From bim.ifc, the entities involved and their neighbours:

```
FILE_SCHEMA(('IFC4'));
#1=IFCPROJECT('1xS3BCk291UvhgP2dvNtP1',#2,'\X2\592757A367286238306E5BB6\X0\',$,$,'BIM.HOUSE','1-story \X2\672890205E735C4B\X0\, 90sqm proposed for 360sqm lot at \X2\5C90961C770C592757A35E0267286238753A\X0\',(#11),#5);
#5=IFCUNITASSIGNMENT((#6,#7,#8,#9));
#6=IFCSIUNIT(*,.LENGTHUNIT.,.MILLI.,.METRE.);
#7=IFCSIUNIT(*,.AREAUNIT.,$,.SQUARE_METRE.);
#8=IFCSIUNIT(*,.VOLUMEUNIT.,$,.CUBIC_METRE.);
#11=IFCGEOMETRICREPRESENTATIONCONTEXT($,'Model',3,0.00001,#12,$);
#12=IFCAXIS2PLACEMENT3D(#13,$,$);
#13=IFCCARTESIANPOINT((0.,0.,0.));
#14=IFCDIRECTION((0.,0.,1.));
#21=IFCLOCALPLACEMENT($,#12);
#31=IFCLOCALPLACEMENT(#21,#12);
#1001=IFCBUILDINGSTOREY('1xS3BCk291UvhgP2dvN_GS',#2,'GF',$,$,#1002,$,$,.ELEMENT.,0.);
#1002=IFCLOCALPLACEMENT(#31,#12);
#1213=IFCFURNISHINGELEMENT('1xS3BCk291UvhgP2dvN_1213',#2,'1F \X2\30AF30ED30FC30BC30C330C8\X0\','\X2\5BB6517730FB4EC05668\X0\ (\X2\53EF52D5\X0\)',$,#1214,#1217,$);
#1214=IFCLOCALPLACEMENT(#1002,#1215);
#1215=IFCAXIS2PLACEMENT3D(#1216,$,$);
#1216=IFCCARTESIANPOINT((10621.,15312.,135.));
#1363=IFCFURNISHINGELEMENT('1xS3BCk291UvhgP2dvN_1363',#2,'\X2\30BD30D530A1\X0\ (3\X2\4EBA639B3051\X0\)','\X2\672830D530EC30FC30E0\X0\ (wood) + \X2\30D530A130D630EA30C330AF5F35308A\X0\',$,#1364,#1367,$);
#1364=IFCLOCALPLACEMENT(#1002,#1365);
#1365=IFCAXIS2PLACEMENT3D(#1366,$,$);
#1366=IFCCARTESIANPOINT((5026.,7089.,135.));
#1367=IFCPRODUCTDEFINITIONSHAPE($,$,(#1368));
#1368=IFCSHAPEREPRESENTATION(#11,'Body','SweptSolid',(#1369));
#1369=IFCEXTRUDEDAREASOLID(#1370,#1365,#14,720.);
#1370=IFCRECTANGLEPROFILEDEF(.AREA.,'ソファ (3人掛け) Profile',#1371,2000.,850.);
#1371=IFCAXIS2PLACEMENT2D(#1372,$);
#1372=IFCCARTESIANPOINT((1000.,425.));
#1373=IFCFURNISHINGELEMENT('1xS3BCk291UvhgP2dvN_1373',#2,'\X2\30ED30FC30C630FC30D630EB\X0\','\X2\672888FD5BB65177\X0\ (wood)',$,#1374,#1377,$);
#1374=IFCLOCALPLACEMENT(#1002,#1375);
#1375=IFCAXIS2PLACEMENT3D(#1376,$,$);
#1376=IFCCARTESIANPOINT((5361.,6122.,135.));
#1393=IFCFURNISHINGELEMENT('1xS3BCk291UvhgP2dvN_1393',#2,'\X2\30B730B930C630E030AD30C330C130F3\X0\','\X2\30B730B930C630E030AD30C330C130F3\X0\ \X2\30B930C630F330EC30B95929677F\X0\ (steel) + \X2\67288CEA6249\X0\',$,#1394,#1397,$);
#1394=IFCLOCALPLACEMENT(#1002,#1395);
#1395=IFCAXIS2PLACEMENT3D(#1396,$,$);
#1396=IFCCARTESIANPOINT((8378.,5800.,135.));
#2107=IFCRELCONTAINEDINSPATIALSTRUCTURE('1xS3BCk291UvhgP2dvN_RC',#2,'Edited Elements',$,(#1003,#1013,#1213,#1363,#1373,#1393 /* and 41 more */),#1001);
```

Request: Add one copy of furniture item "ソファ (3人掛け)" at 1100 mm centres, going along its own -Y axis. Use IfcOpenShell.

```python
import ifcopenshell
import ifcopenshell.api.geometry
import ifcopenshell.api.root
import ifcopenshell.util.element
import ifcopenshell.util.placement
import ifcopenshell.util.unit

model = ifcopenshell.open("bim.ifc")
unit_scale = ifcopenshell.util.unit.calculate_unit_scale(model)


def reuse_history(source, copy):
    """copy_class also copies each property set's owner history, people and application; keep the originals."""
    for rel in copy.IsDefinedBy:
        if rel.is_a("IfcRelDefinesByProperties") and (history := rel.RelatingPropertyDefinition.OwnerHistory):
            rel.RelatingPropertyDefinition.OwnerHistory = source.OwnerHistory
            ifcopenshell.util.element.remove_deep2(model, history)


source = model.by_id(1363)
base = ifcopenshell.util.placement.get_local_placement(source.ObjectPlacement)
step = -base[:3, 1] * 1.1 / unit_scale

for i in range(1, 2):
    copy = ifcopenshell.api.root.copy_class(model, product=source)
    copy.Representation = ifcopenshell.util.element.copy_deep(
        model, source.Representation, exclude=["IfcGeometricRepresentationContext", "IfcRepresentationMap"]
    )
    reuse_history(source, copy)
    matrix = base.copy()
    matrix[:3, 3] += i * step
    print("added at", matrix[:3, 3].round(3) + 0.0)
    ifcopenshell.api.geometry.edit_object_placement(model, product=copy, matrix=matrix, is_si=False)

model.write("bim-out.ifc")
```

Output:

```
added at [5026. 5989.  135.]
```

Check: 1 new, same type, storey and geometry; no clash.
